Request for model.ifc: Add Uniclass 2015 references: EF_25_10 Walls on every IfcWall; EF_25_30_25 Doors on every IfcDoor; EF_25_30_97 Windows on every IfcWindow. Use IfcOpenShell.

First a look at what the model holds.

```python
import ifcopenshell

model = ifcopenshell.open("model.ifc")
print(model.schema)
print("classifications:", [c.Name for c in model.by_type("IfcClassification")])
for ifc_class in ("IfcDoor", "IfcRoof", "IfcStair", "IfcWall", "IfcWindow"):
    print(ifc_class, len(model.by_type(ifc_class)))
```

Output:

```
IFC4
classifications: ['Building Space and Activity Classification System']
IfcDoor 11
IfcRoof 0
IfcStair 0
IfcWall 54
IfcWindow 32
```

```python
import ifcopenshell
import ifcopenshell.api.classification

model = ifcopenshell.open("model.ifc")

system = ifcopenshell.api.classification.add_classification(model, classification="Uniclass 2015")

codes = {
    "IfcWall": ("EF_25_10", "Walls"),
    "IfcDoor": ("EF_25_30_25", "Doors"),
    "IfcWindow": ("EF_25_30_97", "Windows"),
}
for ifc_class, (code, name) in codes.items():
    products = model.by_type(ifc_class)
    ifcopenshell.api.classification.add_reference(
        model, products=products, classification=system, identification=code, name=name
    )
    print(code, len(products))

model.write("model_rev.ifc")
```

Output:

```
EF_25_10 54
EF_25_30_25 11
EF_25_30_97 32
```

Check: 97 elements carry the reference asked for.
